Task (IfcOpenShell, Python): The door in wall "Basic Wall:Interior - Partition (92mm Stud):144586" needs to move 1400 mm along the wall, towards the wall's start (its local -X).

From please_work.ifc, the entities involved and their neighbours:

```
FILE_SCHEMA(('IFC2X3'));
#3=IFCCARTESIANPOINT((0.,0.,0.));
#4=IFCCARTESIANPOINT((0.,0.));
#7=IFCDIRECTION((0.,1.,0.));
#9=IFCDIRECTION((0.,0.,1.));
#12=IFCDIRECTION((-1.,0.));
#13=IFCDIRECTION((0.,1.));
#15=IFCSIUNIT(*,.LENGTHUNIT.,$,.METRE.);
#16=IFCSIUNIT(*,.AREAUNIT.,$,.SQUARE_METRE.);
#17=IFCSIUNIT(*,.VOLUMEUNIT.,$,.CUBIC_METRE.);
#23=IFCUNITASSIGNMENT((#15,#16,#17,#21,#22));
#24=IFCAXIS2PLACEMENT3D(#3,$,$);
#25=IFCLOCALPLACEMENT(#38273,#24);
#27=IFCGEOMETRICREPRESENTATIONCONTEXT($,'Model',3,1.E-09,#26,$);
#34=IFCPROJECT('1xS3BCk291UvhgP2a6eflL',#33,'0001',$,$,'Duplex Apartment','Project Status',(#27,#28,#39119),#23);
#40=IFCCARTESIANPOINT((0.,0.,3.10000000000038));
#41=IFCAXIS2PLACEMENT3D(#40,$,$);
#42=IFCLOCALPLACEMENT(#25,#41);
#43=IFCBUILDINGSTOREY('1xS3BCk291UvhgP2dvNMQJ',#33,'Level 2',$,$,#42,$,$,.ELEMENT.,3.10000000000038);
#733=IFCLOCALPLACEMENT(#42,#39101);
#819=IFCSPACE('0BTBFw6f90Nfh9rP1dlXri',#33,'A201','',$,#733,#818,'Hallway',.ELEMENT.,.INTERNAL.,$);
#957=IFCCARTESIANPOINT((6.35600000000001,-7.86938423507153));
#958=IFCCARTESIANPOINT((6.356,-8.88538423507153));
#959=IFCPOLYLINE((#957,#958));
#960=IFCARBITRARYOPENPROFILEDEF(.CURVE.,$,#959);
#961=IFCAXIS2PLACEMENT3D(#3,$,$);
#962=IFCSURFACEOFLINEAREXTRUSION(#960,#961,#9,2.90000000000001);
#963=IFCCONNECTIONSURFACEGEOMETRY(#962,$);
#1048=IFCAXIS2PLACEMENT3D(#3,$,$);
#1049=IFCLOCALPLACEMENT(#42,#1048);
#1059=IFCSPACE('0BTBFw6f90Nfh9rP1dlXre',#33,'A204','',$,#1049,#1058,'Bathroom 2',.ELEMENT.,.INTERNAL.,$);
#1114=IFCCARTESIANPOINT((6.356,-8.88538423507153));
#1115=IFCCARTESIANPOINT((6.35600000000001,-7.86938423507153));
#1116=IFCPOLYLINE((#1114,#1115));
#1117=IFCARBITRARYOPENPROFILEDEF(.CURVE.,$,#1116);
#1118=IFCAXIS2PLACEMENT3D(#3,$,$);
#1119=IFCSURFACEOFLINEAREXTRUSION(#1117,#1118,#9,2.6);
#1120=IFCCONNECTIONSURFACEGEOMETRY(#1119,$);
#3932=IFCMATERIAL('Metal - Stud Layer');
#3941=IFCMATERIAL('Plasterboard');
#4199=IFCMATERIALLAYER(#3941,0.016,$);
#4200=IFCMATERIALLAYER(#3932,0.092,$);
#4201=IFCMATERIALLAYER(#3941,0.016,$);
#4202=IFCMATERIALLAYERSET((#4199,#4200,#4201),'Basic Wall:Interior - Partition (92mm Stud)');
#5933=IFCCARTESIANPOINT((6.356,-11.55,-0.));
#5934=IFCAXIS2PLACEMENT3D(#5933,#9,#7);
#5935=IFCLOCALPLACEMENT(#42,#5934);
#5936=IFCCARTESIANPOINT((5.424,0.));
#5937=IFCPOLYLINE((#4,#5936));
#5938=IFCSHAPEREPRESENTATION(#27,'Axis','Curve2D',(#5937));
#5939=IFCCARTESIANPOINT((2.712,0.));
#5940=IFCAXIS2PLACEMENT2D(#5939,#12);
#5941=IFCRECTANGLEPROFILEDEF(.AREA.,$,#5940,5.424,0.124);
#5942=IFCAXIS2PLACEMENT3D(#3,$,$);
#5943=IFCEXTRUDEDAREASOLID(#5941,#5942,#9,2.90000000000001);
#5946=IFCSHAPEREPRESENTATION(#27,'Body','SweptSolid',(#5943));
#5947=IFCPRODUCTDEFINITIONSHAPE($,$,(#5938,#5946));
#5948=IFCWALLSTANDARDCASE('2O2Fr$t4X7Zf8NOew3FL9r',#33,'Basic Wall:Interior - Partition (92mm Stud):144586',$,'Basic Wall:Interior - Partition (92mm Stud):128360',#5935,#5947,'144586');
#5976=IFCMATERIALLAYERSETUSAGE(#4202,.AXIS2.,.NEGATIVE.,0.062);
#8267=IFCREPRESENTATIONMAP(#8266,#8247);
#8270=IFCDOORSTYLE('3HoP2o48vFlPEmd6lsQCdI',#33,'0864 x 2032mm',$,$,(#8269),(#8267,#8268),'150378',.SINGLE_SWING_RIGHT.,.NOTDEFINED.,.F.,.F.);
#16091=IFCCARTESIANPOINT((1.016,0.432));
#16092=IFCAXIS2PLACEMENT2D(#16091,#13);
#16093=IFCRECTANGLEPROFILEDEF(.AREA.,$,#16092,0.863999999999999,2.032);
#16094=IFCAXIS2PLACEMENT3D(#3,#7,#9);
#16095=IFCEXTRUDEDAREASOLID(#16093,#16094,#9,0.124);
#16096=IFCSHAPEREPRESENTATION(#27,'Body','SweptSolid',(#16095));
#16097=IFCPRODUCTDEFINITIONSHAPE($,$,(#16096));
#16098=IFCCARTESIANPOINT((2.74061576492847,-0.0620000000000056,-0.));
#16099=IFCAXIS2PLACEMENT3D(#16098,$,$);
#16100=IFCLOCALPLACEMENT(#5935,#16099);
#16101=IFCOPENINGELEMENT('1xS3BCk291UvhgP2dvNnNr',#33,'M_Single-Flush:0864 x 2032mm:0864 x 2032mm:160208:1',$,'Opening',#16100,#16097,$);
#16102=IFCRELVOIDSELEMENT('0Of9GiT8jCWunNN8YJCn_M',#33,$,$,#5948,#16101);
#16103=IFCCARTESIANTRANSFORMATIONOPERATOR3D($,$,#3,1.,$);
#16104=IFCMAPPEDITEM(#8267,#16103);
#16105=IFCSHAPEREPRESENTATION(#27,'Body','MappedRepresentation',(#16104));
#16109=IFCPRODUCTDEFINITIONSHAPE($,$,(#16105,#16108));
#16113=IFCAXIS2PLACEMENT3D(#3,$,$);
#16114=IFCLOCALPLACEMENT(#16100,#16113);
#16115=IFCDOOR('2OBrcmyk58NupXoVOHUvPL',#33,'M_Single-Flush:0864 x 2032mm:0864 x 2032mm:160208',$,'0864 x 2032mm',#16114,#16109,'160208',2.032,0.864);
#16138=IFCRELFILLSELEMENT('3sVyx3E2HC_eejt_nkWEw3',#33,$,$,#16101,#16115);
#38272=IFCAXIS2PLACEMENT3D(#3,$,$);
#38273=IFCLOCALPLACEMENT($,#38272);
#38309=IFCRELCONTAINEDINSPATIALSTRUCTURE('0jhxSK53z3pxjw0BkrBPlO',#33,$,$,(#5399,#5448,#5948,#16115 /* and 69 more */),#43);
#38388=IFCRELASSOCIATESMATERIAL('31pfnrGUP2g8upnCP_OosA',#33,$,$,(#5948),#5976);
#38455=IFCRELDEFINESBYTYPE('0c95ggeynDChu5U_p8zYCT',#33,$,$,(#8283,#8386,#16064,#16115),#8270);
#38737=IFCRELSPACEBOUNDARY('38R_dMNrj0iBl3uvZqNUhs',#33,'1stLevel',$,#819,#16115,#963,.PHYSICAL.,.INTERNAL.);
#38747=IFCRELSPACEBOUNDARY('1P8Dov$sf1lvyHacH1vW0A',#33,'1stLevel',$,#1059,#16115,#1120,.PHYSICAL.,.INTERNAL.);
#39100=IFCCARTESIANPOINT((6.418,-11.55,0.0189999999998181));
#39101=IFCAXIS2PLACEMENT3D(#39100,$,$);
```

```python
import numpy as np
import ifcopenshell
import ifcopenshell.api.geometry
import ifcopenshell.util.placement
import ifcopenshell.util.unit

model = ifcopenshell.open("please_work.ifc")
unit_scale = ifcopenshell.util.unit.calculate_unit_scale(model)

door = model.by_id(16115)
opening = door.FillsVoids[0].RelatingOpeningElement
wall = opening.VoidsElements[0].RelatingBuildingElement

wall_matrix = ifcopenshell.util.placement.get_local_placement(wall.ObjectPlacement)
shift = wall_matrix[:3, 0] * -1.4 / unit_scale
before = ifcopenshell.util.placement.get_local_placement(door.ObjectPlacement)[:3, 3].copy()

# The door is placed relative to its opening, so it follows when the opening moves.
matrix = ifcopenshell.util.placement.get_local_placement(opening.ObjectPlacement)
matrix[:3, 3] += shift
ifcopenshell.api.geometry.edit_object_placement(
    model, product=opening, matrix=matrix, is_si=False, should_transform_children=True
)

# Space boundary surfaces are stored in each space's coordinates; move them too.
for rel in door.ProvidesBoundaries:
    if not rel.ConnectionGeometry:
        continue
    surface = rel.ConnectionGeometry.SurfaceOnRelatingElement
    space_matrix = ifcopenshell.util.placement.get_local_placement(rel.RelatingSpace.ObjectPlacement)
    point = np.array(surface.Position.Location.Coordinates) + space_matrix[:3, :3].T @ shift
    surface.Position = model.createIfcAxis2Placement3D(
        model.createIfcCartesianPoint(point.tolist()), surface.Position.Axis, surface.Position.RefDirection
    )

after = ifcopenshell.util.placement.get_local_placement(door.ObjectPlacement)[:3, 3]
print("door moved by", (after - before).round(3) + 0.0)

model.write("please_work_rev.ifc")
```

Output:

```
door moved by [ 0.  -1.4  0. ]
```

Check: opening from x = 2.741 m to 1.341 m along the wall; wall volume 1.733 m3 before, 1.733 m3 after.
